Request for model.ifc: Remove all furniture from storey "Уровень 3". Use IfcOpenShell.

First a look at what the model holds.

```python
import ifcopenshell
import ifcopenshell.util.element

model = ifcopenshell.open("model.ifc")
print(model.schema)
storey = next(s for s in model.by_type("IfcBuildingStorey") if s.Name == "Уровень 3")
furniture = [e for e in ifcopenshell.util.element.get_decomposition(storey) if e.is_a("IfcFurnishingElement")]
seen = {}
for e in furniture:
    element_type = ifcopenshell.util.element.get_type(e)
    name = element_type.Name if element_type not in (None, e) else None
    seen[name] = seen.get(name, 0) + 1
for name, count in sorted(seen.items(), key=str):
    print(count, "x", name)
```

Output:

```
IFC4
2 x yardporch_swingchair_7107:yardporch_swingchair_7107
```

```python
import ifcopenshell
import ifcopenshell.api.root
import ifcopenshell.util.element

model = ifcopenshell.open("model.ifc")

storey = next(s for s in model.by_type("IfcBuildingStorey") if s.Name == "Уровень 3")
furniture = [e for e in ifcopenshell.util.element.get_decomposition(storey) if e.is_a("IfcFurnishingElement")]

for e in furniture:
    ifcopenshell.api.root.remove_product(model, product=e)
print(len(furniture), "removed")

model.write("model_rev.ifc")
```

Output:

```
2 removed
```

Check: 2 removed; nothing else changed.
